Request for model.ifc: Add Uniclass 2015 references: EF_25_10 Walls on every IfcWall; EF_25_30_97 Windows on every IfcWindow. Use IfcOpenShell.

First a look at what the model holds.

```python
import ifcopenshell

model = ifcopenshell.open("model.ifc")
print(model.schema)
print("classifications:", [c.Name for c in model.by_type("IfcClassification")])
for ifc_class in ("IfcDoor", "IfcRoof", "IfcStair", "IfcWall", "IfcWindow"):
    print(ifc_class, len(model.by_type(ifc_class)))
```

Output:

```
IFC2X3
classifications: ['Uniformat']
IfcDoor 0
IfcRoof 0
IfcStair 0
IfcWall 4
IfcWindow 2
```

```python
import ifcopenshell
import ifcopenshell.api.classification

model = ifcopenshell.open("model.ifc")

# IFC2X3 requires Source and Edition and has no link from the project to the system.
system = model.create_entity("IfcClassification", Source="NBS", Edition="2015", Name="Uniclass 2015")

codes = {
    "IfcWall": ("EF_25_10", "Walls"),
    "IfcWindow": ("EF_25_30_97", "Windows"),
}
for ifc_class, (code, name) in codes.items():
    products = model.by_type(ifc_class)
    ifcopenshell.api.classification.add_reference(
        model, products=products, classification=system, identification=code, name=name
    )
    print(code, len(products))

model.write("model_updated.ifc")
```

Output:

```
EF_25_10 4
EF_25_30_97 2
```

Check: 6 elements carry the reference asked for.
